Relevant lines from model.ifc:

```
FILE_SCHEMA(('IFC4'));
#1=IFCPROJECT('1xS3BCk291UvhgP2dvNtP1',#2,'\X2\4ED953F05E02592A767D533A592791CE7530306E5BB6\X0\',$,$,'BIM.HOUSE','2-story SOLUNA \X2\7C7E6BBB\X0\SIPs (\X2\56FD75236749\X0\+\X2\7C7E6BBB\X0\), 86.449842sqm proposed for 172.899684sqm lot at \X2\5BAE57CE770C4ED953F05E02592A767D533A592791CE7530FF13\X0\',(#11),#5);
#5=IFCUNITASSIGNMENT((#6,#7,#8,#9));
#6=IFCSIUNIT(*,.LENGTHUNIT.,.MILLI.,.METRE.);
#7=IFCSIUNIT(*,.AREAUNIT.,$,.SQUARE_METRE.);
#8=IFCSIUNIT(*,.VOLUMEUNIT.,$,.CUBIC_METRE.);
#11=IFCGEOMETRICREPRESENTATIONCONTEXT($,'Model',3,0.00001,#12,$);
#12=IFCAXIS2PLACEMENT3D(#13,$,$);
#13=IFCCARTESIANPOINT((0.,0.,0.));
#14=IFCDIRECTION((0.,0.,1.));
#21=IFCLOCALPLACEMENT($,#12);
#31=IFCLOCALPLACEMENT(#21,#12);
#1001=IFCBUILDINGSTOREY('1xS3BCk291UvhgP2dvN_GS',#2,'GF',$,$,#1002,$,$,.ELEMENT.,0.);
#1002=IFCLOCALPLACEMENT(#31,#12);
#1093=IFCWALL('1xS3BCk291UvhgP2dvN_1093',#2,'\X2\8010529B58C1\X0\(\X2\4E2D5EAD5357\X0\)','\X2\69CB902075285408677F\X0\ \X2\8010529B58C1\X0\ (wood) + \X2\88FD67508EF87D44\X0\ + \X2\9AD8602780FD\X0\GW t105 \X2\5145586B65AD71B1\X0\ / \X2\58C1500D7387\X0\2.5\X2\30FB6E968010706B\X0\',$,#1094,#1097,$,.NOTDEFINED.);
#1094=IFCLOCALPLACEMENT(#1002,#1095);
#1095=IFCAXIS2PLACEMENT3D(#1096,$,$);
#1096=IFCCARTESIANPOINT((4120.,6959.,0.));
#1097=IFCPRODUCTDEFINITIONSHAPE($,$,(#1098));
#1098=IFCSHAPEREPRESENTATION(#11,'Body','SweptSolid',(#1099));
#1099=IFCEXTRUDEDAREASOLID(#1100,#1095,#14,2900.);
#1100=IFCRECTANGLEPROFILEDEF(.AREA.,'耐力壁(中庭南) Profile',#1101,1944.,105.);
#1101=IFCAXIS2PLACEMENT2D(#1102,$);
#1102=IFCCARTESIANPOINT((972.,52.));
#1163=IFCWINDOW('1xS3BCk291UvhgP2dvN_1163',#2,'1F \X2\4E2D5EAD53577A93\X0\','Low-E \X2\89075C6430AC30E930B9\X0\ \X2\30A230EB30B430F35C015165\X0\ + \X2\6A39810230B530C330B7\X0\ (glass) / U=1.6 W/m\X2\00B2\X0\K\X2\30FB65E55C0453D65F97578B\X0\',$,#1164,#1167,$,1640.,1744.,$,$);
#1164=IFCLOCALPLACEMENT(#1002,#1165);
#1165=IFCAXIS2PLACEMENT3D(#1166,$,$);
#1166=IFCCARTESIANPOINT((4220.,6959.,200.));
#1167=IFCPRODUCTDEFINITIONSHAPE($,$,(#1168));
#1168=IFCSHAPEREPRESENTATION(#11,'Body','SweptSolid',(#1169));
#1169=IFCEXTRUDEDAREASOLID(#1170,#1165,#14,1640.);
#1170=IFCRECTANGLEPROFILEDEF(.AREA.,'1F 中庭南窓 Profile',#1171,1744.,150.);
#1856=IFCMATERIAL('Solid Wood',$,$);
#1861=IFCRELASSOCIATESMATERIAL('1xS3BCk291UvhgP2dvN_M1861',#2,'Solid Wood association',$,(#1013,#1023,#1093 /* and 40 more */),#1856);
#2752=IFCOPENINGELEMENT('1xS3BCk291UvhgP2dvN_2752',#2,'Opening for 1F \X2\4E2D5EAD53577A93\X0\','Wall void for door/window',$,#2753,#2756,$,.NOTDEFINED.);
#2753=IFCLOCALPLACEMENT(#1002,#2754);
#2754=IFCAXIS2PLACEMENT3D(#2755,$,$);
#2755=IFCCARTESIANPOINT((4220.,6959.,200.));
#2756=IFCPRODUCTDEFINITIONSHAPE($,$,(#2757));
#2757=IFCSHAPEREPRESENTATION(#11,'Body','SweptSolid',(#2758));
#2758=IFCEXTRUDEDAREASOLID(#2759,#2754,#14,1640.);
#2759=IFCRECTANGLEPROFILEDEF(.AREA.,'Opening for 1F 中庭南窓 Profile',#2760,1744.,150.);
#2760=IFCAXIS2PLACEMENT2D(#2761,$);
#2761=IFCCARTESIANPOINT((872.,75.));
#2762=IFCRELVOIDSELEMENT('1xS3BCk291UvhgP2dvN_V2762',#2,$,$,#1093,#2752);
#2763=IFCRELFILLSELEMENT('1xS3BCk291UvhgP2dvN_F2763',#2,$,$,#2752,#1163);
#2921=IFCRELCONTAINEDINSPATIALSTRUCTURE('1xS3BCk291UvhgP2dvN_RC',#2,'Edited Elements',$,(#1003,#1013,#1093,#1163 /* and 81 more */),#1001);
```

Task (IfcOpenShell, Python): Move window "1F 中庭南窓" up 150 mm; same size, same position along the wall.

```python
import numpy as np
import ifcopenshell
import ifcopenshell.api.geometry
import ifcopenshell.util.placement
import ifcopenshell.util.unit

model = ifcopenshell.open("model.ifc")
unit_scale = ifcopenshell.util.unit.calculate_unit_scale(model)

window = model.by_id(1163)
opening = window.FillsVoids[0].RelatingOpeningElement
dz = 0.15 / unit_scale

shift = np.array([0.0, 0.0, dz])
# The window is not placed relative to its opening, so move both.
for product in (opening, window):
    matrix = ifcopenshell.util.placement.get_local_placement(product.ObjectPlacement)
    matrix[:3, 3] += shift
    ifcopenshell.api.geometry.edit_object_placement(model, product=product, matrix=matrix, is_si=False)

print(f"moved by {dz * unit_scale:+.3f} m")

model.write("model_rev.ifc")
```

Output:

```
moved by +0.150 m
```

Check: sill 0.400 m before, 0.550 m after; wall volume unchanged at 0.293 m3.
